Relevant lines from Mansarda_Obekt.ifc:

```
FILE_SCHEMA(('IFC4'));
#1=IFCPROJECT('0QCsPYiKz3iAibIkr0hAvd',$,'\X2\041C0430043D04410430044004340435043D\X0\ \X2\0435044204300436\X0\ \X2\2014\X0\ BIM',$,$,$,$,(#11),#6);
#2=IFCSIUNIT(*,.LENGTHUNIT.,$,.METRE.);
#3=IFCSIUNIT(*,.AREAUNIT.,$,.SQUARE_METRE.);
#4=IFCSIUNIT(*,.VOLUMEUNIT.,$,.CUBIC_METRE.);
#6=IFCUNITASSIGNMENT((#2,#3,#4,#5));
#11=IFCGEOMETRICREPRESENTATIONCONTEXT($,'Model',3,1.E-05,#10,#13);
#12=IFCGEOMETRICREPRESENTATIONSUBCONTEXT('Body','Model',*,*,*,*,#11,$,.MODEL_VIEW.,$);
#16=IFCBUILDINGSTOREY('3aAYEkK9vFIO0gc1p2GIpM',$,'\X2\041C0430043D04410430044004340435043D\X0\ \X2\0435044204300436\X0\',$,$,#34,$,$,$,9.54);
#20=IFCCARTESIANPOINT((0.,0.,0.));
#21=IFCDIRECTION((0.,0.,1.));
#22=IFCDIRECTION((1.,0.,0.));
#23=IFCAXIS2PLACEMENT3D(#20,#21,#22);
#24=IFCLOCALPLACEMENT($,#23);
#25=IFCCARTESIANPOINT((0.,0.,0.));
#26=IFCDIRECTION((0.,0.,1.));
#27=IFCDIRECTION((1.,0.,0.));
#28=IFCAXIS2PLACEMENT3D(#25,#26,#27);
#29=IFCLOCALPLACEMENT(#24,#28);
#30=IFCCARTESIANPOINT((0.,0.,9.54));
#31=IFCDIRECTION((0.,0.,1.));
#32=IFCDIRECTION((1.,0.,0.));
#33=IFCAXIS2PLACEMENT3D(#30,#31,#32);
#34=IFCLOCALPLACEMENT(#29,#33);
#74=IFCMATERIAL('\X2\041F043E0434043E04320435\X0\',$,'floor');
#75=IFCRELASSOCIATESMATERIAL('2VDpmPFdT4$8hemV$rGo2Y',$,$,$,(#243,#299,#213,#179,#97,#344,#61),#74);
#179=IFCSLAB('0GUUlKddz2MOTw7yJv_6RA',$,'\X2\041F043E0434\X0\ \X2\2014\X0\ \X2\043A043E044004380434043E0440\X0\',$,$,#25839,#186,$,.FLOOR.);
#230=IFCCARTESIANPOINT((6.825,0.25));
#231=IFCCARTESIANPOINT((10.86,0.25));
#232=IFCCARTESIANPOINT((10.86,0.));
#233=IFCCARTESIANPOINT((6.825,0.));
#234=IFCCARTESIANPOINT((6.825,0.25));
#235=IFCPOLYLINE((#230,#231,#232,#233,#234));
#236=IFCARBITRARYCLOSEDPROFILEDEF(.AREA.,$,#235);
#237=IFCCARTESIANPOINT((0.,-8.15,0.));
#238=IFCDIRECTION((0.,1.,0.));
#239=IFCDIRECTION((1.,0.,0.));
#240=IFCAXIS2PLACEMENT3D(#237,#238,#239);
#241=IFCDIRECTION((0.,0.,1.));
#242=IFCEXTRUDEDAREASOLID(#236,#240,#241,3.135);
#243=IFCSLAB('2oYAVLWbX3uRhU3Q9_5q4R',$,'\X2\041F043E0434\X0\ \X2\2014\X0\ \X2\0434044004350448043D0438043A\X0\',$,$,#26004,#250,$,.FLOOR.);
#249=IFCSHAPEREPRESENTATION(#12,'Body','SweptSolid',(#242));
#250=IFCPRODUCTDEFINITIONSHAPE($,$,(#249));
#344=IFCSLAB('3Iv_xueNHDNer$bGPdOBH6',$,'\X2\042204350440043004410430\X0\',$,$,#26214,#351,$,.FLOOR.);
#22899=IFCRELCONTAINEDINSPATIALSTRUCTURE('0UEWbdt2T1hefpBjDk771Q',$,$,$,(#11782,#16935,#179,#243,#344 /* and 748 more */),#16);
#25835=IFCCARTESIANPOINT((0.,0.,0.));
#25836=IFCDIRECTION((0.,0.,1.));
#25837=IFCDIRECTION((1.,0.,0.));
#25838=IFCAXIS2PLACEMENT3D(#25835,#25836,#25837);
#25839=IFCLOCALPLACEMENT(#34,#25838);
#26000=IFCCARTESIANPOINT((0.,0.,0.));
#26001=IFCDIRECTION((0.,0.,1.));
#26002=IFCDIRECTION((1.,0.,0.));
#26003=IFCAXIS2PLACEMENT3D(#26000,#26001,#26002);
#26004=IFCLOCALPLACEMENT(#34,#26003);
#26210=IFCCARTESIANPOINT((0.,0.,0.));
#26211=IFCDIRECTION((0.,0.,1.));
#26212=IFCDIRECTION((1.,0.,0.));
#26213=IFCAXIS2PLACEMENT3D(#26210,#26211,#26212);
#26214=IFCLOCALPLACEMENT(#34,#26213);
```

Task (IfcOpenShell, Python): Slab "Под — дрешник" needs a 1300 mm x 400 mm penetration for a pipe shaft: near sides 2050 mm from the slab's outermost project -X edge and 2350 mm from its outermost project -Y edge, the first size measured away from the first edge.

```python
import numpy as np
import ifcopenshell
import ifcopenshell.api.feature
import ifcopenshell.api.geometry
import ifcopenshell.api.root
import ifcopenshell.geom
import ifcopenshell.util.placement
import ifcopenshell.util.representation
import ifcopenshell.util.shape
import ifcopenshell.util.unit

model = ifcopenshell.open("Mansarda_Obekt.ifc")
unit_scale = ifcopenshell.util.unit.calculate_unit_scale(model)
settings = ifcopenshell.geom.settings()


def volume(element):
    """Net volume in cubic metres, openings subtracted."""
    shape = ifcopenshell.geom.create_shape(settings, element)
    return ifcopenshell.util.shape.get_volume(shape.geometry)


slab = model.by_guid("2oYAVLWbX3uRhU3Q9_5q4R")
before = volume(slab)

# Extent in the slab's own axes, in metres. The edges named are its -X and -Y sides.
slab_shape = ifcopenshell.geom.create_shape(settings, slab)
vertices = ifcopenshell.util.shape.get_vertices(slab_shape.geometry)
x_min, y_min, bottom = vertices.min(axis=0)
top = vertices[:, 2].max()

opening = ifcopenshell.api.root.create_entity(model, ifc_class="IfcOpeningElement", name="Pipe shaft opening", predefined_type="OPENING")
context = ifcopenshell.util.representation.get_context(model, "Model", "Body", "MODEL_VIEW")
width, depth = 1.3, 0.4
outline = [(0.0, 0.0), (width, 0.0), (width, depth), (0.0, depth), (0.0, 0.0)]
# Overshoot both faces by 50 mm so the cut is clean.
shape = ifcopenshell.api.geometry.add_slab_representation(
    model, context=context, depth=top - bottom + 0.1, polyline=outline
)
ifcopenshell.api.geometry.assign_representation(model, product=opening, representation=shape)

matrix = ifcopenshell.util.placement.get_local_placement(slab.ObjectPlacement)
matrix[:, 3] = matrix @ np.append(np.array([x_min + 2.05, y_min + 2.35, bottom - 0.05]) / unit_scale, 1.0)
ifcopenshell.api.geometry.edit_object_placement(model, product=opening, matrix=matrix, is_si=False)
ifcopenshell.api.feature.add_feature(model, feature=opening, element=slab)

after = volume(slab)

print(f"slab volume {before:.3f} -> {after:.3f} m3")

model.write("Mansarda_Obekt-out.ifc")
```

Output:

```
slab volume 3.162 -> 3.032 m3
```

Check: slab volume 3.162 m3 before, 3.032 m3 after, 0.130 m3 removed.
